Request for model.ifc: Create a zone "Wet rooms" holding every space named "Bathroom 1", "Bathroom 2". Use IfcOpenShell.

First a look at what the model holds.

```python
import ifcopenshell

model = ifcopenshell.open("model.ifc")
print(model.schema)
seen = {}
for space in model.by_type("IfcSpace"):
    seen[space.LongName] = seen.get(space.LongName, 0) + 1
for name, count in sorted(seen.items(), key=str):
    print(count, "x", name)
print("zones:", [z.Name for z in model.by_type("IfcZone")][:20])
```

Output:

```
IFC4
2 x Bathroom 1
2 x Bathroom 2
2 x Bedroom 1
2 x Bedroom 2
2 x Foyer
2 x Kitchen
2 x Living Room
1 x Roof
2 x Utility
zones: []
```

```python
import ifcopenshell
import ifcopenshell.api.group
import ifcopenshell.api.root

model = ifcopenshell.open("model.ifc")

names = {"Bathroom 1", "Bathroom 2"}
spaces = [s for s in model.by_type("IfcSpace") if s.LongName in names]

zone = ifcopenshell.api.root.create_entity(model, ifc_class="IfcZone", name="Wet rooms")
ifcopenshell.api.group.assign_group(model, products=spaces, group=zone)
print(len(spaces), "spaces in", zone.Name)

model.write("model_rev.ifc")
```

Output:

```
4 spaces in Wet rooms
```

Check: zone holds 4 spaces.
